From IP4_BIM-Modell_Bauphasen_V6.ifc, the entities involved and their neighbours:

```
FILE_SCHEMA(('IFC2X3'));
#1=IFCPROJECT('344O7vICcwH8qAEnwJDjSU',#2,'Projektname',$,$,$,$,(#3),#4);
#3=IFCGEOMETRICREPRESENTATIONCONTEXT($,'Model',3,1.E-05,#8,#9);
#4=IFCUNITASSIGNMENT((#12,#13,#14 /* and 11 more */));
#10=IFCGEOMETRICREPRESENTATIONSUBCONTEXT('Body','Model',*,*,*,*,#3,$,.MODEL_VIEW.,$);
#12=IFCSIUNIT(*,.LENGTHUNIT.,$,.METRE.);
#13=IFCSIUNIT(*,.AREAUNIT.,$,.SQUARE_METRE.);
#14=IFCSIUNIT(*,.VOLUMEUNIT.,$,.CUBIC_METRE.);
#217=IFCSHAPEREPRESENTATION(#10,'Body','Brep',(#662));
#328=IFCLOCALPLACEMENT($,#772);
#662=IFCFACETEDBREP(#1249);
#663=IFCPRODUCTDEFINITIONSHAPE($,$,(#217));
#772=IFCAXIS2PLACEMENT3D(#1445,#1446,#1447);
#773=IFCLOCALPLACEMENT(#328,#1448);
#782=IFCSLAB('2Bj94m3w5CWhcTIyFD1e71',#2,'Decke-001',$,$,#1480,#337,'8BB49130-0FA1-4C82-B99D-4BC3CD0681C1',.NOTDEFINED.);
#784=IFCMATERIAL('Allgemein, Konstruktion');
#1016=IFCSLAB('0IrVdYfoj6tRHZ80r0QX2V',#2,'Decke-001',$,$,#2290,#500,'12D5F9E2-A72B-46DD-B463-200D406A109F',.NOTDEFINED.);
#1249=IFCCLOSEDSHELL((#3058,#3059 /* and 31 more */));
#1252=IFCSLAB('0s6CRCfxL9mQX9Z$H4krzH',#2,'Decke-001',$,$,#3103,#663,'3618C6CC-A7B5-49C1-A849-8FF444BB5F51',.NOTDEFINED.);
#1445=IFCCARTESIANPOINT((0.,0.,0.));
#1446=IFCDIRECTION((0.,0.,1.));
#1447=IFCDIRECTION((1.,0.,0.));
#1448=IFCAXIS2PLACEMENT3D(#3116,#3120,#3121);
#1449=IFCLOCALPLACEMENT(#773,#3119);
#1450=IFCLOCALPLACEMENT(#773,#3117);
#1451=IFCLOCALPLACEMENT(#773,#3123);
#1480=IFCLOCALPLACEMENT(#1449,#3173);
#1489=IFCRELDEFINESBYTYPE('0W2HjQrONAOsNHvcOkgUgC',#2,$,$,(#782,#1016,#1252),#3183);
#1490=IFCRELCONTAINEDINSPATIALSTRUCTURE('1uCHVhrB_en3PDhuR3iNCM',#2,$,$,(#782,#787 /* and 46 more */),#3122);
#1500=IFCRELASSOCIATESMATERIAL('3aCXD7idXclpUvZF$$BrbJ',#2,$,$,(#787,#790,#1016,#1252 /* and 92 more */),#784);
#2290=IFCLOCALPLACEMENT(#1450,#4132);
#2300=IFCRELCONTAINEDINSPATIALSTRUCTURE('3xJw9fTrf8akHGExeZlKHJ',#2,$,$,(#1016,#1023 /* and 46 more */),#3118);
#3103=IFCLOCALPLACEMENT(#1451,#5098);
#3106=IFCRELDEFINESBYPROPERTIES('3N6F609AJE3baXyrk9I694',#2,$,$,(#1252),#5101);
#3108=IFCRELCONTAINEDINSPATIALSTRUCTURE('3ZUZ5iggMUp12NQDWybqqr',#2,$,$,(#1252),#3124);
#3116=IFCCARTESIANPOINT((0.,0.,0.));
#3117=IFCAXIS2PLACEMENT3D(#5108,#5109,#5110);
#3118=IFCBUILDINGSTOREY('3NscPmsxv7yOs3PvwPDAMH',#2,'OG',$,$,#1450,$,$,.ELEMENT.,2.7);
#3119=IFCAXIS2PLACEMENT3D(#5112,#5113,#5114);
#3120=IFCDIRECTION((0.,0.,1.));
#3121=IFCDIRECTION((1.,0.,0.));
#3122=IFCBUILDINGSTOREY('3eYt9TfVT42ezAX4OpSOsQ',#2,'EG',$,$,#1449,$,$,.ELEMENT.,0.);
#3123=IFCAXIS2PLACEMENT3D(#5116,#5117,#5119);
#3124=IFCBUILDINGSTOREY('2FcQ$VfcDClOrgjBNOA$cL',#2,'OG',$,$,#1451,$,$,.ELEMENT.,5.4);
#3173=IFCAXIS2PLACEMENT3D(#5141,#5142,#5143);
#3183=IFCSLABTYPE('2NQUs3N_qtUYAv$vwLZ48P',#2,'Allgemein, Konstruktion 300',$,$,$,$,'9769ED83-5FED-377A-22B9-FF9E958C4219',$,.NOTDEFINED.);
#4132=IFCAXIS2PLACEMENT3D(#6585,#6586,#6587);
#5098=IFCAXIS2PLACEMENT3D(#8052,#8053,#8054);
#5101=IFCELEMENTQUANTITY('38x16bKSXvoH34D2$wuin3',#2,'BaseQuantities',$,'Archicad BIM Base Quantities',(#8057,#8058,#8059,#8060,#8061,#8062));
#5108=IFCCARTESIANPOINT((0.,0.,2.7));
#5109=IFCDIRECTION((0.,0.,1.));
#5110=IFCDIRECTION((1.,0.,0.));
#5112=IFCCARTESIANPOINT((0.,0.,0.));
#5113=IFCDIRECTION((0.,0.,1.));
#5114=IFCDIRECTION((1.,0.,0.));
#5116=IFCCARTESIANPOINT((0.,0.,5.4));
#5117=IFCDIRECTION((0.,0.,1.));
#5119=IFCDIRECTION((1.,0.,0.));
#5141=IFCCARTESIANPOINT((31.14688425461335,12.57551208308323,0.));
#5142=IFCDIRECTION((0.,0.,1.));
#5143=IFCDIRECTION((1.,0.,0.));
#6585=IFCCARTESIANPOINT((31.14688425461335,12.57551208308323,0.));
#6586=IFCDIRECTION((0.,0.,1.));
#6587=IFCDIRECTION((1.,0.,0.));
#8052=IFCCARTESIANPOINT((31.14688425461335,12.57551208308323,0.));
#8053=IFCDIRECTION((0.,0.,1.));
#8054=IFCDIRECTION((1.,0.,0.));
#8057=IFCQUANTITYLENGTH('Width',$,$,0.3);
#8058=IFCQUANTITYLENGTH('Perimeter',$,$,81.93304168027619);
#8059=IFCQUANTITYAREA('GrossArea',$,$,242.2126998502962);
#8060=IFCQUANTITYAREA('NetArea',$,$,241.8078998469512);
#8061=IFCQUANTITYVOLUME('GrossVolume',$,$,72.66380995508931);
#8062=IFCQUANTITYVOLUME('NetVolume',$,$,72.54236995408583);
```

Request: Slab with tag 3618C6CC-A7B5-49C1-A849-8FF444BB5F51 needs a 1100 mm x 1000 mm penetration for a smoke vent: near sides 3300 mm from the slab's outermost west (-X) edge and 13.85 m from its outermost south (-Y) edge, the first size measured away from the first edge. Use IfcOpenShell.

```python
import numpy as np
import ifcopenshell
import ifcopenshell.api.feature
import ifcopenshell.api.geometry
import ifcopenshell.api.pset
import ifcopenshell.api.root
import ifcopenshell.geom
import ifcopenshell.util.element
import ifcopenshell.util.placement
import ifcopenshell.util.representation
import ifcopenshell.util.shape
import ifcopenshell.util.unit

model = ifcopenshell.open("IP4_BIM-Modell_Bauphasen_V6.ifc")
unit_scale = ifcopenshell.util.unit.calculate_unit_scale(model)
area_scale = ifcopenshell.util.unit.calculate_unit_scale(model, "AREAUNIT")
volume_scale = ifcopenshell.util.unit.calculate_unit_scale(model, "VOLUMEUNIT")
settings = ifcopenshell.geom.settings()


def volume(element):
    """Net volume in cubic metres, openings subtracted."""
    shape = ifcopenshell.geom.create_shape(settings, element)
    return ifcopenshell.util.shape.get_volume(shape.geometry)


slab = model.by_guid("0s6CRCfxL9mQX9Z$H4krzH")
before = volume(slab)

# Extent in the slab's own axes, in metres. The edges named are its -X and -Y sides.
slab_shape = ifcopenshell.geom.create_shape(settings, slab)
vertices = ifcopenshell.util.shape.get_vertices(slab_shape.geometry)
x_min, y_min, bottom = vertices.min(axis=0)
top = vertices[:, 2].max()

opening = ifcopenshell.api.root.create_entity(model, ifc_class="IfcOpeningElement", name="Smoke vent opening")
context = ifcopenshell.util.representation.get_context(model, "Model", "Body", "MODEL_VIEW")
width, depth = 1.1, 1
outline = [(0.0, 0.0), (width, 0.0), (width, depth), (0.0, depth), (0.0, 0.0)]
# Overshoot both faces by 50 mm so the cut is clean.
shape = ifcopenshell.api.geometry.add_slab_representation(
    model, context=context, depth=top - bottom + 0.1, polyline=outline
)
ifcopenshell.api.geometry.assign_representation(model, product=opening, representation=shape)

matrix = ifcopenshell.util.placement.get_local_placement(slab.ObjectPlacement)
matrix[:, 3] = matrix @ np.append(np.array([x_min + 3.3, y_min + 13.85, bottom - 0.05]) / unit_scale, 1.0)
ifcopenshell.api.geometry.edit_object_placement(model, product=opening, matrix=matrix, is_si=False)
ifcopenshell.api.feature.add_feature(model, feature=opening, element=slab)

after = volume(slab)

# Update the slab's stored quantities.
qto = model.by_id(ifcopenshell.util.element.get_pset(slab, "BaseQuantities", should_inherit=False)["id"])
ifcopenshell.api.pset.edit_qto(model, qto=qto, properties={
    "NetArea": after / (top - bottom) / area_scale,
    "NetVolume": after / volume_scale,
})

print(f"slab volume {before:.3f} -> {after:.3f} m3")

model.write("IP4_BIM-Modell_Bauphasen_V6_updated.ifc")
```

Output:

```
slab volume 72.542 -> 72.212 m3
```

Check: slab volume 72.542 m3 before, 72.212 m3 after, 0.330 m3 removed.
